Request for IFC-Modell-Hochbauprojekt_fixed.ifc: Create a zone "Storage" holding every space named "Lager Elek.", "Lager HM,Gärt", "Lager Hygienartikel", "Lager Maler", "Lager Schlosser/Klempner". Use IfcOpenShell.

First a look at what the model holds.

```python
import ifcopenshell

model = ifcopenshell.open("IFC-Modell-Hochbauprojekt_fixed.ifc")
print(model.schema)
seen = {}
for space in model.by_type("IfcSpace"):
    seen[space.LongName] = seen.get(space.LongName, 0) + 1
for name, count in sorted(seen.items(), key=str):
    print(count, "x", name)
print("zones:", [z.Name for z in model.by_type("IfcZone")][:20])
```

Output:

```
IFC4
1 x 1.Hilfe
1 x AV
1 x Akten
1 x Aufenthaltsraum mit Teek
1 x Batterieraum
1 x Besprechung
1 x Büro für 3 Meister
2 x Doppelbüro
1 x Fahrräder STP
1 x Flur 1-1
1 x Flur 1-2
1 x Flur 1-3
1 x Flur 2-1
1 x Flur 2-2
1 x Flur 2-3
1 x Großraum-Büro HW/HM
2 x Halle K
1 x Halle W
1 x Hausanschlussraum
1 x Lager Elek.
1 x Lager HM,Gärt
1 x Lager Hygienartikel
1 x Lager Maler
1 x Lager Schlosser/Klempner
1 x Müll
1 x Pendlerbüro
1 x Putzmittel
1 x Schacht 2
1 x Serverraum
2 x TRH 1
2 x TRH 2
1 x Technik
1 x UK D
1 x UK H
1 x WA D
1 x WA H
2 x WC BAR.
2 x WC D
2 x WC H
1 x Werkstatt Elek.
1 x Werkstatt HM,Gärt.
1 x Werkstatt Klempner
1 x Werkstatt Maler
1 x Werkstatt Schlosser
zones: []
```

```python
import ifcopenshell
import ifcopenshell.api.group
import ifcopenshell.api.root

model = ifcopenshell.open("IFC-Modell-Hochbauprojekt_fixed.ifc")

names = {"Lager Elek.", "Lager HM,Gärt", "Lager Hygienartikel", "Lager Maler", "Lager Schlosser/Klempner"}
spaces = [s for s in model.by_type("IfcSpace") if s.LongName in names]

zone = ifcopenshell.api.root.create_entity(model, ifc_class="IfcZone", name="Storage")
ifcopenshell.api.group.assign_group(model, products=spaces, group=zone)
print(len(spaces), "spaces in", zone.Name)

model.write("IFC-Modell-Hochbauprojekt_fixed_updated.ifc")
```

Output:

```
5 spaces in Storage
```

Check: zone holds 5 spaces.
